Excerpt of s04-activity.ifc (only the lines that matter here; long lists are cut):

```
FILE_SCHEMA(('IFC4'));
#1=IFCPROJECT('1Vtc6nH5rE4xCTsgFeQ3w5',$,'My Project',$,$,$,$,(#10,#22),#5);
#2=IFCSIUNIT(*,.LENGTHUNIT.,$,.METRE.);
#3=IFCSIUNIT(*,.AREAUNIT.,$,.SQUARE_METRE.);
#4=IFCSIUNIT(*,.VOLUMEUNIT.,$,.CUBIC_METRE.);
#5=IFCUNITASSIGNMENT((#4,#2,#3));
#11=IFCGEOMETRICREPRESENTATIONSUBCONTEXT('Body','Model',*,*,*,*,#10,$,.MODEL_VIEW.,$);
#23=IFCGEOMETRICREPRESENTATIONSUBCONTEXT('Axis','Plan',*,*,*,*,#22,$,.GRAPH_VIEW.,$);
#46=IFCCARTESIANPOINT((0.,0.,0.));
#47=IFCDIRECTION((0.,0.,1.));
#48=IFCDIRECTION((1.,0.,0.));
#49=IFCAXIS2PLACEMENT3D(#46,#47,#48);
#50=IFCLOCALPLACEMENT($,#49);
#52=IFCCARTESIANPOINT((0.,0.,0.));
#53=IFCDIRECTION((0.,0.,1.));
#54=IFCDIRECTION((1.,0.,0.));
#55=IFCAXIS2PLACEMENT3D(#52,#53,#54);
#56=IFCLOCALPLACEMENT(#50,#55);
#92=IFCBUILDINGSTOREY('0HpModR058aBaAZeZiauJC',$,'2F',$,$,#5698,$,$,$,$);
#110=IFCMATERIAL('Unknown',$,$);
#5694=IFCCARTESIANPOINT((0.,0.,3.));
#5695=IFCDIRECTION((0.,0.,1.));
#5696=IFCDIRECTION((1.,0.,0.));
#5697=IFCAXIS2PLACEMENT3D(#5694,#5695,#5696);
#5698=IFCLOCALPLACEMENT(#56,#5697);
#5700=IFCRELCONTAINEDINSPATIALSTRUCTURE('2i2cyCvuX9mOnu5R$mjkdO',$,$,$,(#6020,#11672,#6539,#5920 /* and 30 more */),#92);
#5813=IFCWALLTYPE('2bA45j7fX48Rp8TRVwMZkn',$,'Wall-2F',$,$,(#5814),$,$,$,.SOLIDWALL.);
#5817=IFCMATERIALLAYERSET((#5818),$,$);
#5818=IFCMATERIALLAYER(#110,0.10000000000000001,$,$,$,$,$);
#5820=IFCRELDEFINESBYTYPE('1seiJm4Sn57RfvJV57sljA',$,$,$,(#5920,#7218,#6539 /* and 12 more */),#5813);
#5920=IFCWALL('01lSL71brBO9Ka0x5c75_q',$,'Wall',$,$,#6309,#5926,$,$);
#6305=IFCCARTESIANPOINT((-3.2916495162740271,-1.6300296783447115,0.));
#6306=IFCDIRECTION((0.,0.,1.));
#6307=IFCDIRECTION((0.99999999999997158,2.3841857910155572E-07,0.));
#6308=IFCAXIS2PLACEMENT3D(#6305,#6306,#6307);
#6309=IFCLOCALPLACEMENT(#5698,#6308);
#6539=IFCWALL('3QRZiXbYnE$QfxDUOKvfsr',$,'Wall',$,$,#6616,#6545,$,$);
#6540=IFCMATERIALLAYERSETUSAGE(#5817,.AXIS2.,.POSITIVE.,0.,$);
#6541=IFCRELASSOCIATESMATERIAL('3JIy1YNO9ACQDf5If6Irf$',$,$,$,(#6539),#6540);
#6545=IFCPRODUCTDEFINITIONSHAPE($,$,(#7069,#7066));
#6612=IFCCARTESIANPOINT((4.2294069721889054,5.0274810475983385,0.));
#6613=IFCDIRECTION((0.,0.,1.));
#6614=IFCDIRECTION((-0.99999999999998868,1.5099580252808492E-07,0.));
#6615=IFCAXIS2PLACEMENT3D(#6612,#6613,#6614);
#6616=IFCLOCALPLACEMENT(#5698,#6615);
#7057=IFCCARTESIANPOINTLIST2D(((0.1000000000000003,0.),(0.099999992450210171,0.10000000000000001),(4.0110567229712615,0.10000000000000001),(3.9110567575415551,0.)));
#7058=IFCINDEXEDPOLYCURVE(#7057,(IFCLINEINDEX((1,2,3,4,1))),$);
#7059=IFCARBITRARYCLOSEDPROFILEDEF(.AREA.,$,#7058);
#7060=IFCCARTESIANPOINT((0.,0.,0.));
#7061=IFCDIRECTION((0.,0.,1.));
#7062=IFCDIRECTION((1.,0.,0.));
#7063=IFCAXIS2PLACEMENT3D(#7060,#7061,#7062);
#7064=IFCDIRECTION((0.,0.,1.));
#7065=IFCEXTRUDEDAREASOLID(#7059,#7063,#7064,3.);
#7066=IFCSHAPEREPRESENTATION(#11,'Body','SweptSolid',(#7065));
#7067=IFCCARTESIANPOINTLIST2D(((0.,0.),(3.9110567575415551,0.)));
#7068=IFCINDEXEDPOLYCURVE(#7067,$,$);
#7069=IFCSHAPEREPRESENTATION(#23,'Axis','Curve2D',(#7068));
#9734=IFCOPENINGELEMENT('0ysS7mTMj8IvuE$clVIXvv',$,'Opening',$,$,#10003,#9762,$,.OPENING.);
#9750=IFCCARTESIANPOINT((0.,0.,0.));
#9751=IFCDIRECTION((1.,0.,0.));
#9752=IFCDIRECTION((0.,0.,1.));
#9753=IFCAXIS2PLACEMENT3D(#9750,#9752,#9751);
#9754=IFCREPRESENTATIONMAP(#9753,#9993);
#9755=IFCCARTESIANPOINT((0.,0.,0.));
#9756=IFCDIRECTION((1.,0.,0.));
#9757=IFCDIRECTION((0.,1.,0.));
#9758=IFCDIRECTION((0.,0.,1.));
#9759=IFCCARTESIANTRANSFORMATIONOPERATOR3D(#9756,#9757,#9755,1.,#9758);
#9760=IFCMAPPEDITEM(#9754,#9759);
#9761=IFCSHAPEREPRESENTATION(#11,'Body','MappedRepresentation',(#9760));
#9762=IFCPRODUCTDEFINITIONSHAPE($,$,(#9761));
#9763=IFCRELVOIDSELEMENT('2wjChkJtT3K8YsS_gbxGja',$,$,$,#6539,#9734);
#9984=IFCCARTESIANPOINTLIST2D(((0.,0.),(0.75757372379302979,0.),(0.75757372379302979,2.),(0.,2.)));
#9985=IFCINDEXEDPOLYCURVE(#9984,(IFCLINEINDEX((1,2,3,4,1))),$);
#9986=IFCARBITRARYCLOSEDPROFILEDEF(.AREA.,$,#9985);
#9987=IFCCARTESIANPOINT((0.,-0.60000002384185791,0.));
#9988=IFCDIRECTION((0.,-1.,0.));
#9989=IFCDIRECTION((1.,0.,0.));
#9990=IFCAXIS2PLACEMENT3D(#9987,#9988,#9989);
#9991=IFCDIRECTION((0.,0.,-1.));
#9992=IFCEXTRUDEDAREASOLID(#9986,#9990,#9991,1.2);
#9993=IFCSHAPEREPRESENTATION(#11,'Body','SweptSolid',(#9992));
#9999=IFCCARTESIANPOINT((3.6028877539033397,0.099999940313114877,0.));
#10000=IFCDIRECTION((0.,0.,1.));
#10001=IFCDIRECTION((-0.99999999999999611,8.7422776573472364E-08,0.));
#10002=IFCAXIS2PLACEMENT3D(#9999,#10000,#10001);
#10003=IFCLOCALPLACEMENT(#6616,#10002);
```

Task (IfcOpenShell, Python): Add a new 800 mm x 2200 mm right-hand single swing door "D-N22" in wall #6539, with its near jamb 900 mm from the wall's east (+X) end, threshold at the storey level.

```python
import numpy as np
import ifcopenshell
import ifcopenshell.api.feature
import ifcopenshell.api.geometry
import ifcopenshell.api.root
import ifcopenshell.api.spatial
import ifcopenshell.geom
import ifcopenshell.util.element
import ifcopenshell.util.placement
import ifcopenshell.util.representation
import ifcopenshell.util.shape
import ifcopenshell.util.unit

model = ifcopenshell.open("s04-activity.ifc")
unit_scale = ifcopenshell.util.unit.calculate_unit_scale(model)
settings = ifcopenshell.geom.settings()


def volume(element):
    """Net volume in cubic metres, openings subtracted."""
    shape = ifcopenshell.geom.create_shape(settings, element)
    return ifcopenshell.util.shape.get_volume(shape.geometry)


wall = model.by_guid("3QRZiXbYnE$QfxDUOKvfsr")
storey = ifcopenshell.util.element.get_container(wall, ifc_class="IfcBuildingStorey")
context = ifcopenshell.util.representation.get_context(model, "Model", "Body", "MODEL_VIEW")
before = volume(wall)

width, height, from_end, sill = 0.8, 2.2, 0.9, 0.0  # metres

# The wall runs along its own X axis, and the end named is its -X end.
wall_shape = ifcopenshell.geom.create_shape(settings, wall)
x, y, z = ifcopenshell.util.shape.get_vertices(wall_shape.geometry).T
start = x.min() + from_end
face, thickness = float(y.min()), float(y.max() - y.min())
wall_matrix = ifcopenshell.util.placement.get_local_placement(wall.ObjectPlacement)
level = ifcopenshell.util.placement.get_local_placement(storey.ObjectPlacement)[2, 3]


def in_wall(x, y):
    """Placement at x, y metres in the wall's axes, at sill height."""
    matrix = wall_matrix.copy()
    matrix[:, 3] = wall_matrix @ np.array([x / unit_scale, y / unit_scale, 0.0, 1.0])
    matrix[2, 3] = level + sill / unit_scale
    return matrix


# Opening: a box that overshoots both wall faces by 50 mm.
opening = ifcopenshell.api.root.create_entity(model, ifc_class="IfcOpeningElement", predefined_type="OPENING")
box = ifcopenshell.api.geometry.add_wall_representation(
    model, context=context, length=width, height=height, thickness=thickness + 0.1
)
ifcopenshell.api.geometry.assign_representation(model, product=opening, representation=box)
ifcopenshell.api.geometry.edit_object_placement(model, product=opening, matrix=in_wall(start, face - 0.05), is_si=False)
ifcopenshell.api.feature.add_feature(model, feature=opening, element=wall)

door = ifcopenshell.api.root.create_entity(model, ifc_class="IfcDoor", name="D-N22", predefined_type="DOOR")
door.OverallWidth, door.OverallHeight = width / unit_scale, height / unit_scale
door.OperationType = "SINGLE_SWING_RIGHT"
body = ifcopenshell.api.geometry.add_door_representation(
    model,
    context=context,
    overall_width=door.OverallWidth,
    overall_height=door.OverallHeight,
    operation_type="SINGLE_SWING_RIGHT",
    lining_properties={"LiningDepth": thickness / unit_scale, "ThresholdDepth": thickness / unit_scale},
)
ifcopenshell.api.geometry.assign_representation(model, product=door, representation=body)
ifcopenshell.api.spatial.assign_container(model, products=[door], relating_structure=storey)
ifcopenshell.api.feature.add_filling(model, opening=opening, element=door)

# The lining spans the wall, so the door starts at the wall face.
ifcopenshell.api.geometry.edit_object_placement(model, product=door, matrix=in_wall(start, face), is_si=False)

after = volume(wall)

print(f"wall volume {before:.3f} -> {after:.3f} m3")

model.write("s04-activity_edited.ifc")
```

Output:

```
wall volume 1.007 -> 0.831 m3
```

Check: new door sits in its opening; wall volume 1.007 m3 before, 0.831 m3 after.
